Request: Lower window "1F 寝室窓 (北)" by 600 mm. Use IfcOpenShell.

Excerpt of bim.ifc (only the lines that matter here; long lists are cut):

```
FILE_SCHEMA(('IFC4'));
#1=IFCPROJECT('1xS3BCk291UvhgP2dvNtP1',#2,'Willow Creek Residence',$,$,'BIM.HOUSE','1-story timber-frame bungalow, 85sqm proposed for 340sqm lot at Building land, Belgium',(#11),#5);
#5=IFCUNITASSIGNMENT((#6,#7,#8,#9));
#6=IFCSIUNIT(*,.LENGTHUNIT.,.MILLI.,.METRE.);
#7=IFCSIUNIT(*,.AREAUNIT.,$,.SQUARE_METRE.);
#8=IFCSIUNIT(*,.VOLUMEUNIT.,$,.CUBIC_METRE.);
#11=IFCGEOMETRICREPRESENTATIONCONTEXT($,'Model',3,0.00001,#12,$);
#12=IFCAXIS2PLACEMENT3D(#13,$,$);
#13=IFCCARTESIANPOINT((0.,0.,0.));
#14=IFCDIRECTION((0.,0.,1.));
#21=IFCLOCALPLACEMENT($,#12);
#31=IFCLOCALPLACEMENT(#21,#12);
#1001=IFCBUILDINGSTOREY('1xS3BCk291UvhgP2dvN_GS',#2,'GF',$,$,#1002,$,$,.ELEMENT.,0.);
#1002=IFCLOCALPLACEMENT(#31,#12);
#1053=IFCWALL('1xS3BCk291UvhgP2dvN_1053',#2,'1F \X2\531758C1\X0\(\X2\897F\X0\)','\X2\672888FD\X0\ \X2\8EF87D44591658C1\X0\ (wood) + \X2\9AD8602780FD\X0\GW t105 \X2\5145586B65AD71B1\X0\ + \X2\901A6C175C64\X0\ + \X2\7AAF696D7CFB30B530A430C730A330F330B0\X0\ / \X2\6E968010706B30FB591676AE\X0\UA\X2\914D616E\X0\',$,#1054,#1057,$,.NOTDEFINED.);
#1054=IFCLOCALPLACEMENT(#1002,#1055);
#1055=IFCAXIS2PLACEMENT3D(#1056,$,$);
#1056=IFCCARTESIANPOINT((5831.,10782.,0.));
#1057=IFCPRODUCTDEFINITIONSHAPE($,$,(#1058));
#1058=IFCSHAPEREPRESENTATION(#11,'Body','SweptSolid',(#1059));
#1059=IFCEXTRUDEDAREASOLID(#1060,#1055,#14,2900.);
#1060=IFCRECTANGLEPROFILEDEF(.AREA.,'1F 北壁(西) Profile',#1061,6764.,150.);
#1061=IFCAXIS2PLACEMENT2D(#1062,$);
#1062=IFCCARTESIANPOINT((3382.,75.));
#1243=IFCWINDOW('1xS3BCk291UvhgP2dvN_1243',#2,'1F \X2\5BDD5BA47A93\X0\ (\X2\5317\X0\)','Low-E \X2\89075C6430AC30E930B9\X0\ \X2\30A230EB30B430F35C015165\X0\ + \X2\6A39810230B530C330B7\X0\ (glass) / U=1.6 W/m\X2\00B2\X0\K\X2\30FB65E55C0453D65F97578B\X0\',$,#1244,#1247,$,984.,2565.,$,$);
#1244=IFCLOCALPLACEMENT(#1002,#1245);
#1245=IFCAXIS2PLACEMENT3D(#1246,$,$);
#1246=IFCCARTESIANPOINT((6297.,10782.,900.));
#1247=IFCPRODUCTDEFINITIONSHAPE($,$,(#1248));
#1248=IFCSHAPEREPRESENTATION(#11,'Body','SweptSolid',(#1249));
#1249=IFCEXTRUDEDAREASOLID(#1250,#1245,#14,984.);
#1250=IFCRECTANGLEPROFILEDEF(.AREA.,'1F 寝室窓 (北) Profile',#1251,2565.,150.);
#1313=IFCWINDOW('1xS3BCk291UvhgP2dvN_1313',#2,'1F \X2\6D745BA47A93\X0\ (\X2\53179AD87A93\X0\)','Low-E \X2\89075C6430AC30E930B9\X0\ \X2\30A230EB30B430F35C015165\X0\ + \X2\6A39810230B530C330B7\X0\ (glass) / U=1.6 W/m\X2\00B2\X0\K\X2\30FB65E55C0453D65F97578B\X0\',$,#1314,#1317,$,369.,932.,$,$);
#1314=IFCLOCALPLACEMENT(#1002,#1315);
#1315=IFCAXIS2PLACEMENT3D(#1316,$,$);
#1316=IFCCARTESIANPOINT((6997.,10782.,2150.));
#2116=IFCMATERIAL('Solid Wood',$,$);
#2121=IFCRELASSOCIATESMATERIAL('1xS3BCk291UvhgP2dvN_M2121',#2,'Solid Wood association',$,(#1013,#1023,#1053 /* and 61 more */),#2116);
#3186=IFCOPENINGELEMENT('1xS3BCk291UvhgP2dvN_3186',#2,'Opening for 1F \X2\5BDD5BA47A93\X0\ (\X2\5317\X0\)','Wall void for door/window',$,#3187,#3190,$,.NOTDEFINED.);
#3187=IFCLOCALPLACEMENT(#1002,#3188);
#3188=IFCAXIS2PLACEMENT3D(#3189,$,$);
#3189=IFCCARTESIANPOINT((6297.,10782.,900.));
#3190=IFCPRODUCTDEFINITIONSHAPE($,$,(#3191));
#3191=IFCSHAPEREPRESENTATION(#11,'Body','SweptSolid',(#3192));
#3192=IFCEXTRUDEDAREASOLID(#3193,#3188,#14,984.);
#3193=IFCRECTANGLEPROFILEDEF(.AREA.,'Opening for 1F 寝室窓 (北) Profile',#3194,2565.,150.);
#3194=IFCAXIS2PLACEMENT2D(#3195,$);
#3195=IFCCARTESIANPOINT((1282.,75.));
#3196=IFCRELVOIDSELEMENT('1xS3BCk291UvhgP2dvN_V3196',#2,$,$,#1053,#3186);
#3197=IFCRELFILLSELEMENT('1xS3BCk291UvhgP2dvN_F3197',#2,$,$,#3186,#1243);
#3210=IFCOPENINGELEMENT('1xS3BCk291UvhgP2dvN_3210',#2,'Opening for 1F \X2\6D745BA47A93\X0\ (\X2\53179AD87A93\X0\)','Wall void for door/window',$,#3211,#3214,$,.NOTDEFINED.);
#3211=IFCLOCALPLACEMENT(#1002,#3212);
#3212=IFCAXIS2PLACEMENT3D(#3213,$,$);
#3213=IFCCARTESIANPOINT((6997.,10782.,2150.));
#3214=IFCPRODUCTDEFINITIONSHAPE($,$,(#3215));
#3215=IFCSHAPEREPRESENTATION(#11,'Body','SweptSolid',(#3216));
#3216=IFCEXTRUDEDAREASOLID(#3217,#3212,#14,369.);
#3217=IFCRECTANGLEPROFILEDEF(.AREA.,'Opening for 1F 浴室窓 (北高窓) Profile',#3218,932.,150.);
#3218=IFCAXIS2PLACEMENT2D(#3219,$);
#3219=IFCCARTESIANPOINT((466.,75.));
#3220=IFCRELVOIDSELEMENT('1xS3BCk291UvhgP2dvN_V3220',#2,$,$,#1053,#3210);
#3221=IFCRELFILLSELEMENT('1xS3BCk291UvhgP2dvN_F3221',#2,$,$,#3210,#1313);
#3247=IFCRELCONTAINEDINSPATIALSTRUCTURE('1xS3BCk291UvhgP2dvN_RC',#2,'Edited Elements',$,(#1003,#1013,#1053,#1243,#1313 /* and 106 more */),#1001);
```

```python
import numpy as np
import ifcopenshell
import ifcopenshell.api.geometry
import ifcopenshell.util.placement
import ifcopenshell.util.unit

model = ifcopenshell.open("bim.ifc")
unit_scale = ifcopenshell.util.unit.calculate_unit_scale(model)

window = model.by_guid("1xS3BCk291UvhgP2dvN_1243")
opening = window.FillsVoids[0].RelatingOpeningElement
dz = -0.6 / unit_scale

shift = np.array([0.0, 0.0, dz])
# The window is not placed relative to its opening, so move both.
for product in (opening, window):
    matrix = ifcopenshell.util.placement.get_local_placement(product.ObjectPlacement)
    matrix[:3, 3] += shift
    ifcopenshell.api.geometry.edit_object_placement(model, product=product, matrix=matrix, is_si=False)

print(f"moved by {dz * unit_scale:+.3f} m")

model.write("bim-out.ifc")
```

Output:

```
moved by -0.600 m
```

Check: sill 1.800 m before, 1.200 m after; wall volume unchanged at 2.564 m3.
